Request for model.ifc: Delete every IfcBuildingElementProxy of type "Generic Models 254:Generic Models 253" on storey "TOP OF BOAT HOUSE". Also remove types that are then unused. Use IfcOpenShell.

First a look at what the model holds.

```python
import ifcopenshell
import ifcopenshell.util.element

model = ifcopenshell.open("model.ifc")
print(model.schema)
storey = next(s for s in model.by_type("IfcBuildingStorey") if s.Name == "TOP OF BOAT HOUSE")
proxies = [e for e in ifcopenshell.util.element.get_decomposition(storey) if e.is_a("IfcBuildingElementProxy")]
seen = {}
for e in proxies:
    element_type = ifcopenshell.util.element.get_type(e)
    name = element_type.Name if element_type not in (None, e) else None
    seen[name] = seen.get(name, 0) + 1
for name, count in sorted(seen.items(), key=str):
    print(count, "x", name)
```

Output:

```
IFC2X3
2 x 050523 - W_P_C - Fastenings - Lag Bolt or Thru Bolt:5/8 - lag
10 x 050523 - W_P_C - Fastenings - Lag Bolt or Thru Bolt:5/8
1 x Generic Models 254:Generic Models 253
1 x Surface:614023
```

```python
import ifcopenshell
import ifcopenshell.api.root
import ifcopenshell.util.element

model = ifcopenshell.open("model.ifc")

storey = next(s for s in model.by_type("IfcBuildingStorey") if s.Name == "TOP OF BOAT HOUSE")
proxies = [e for e in ifcopenshell.util.element.get_decomposition(storey) if e.is_a("IfcBuildingElementProxy")]
targets = [e for e in proxies if (t := ifcopenshell.util.element.get_type(e)) not in (None, e) and t.Name == "Generic Models 254:Generic Models 253"]
types = {ifcopenshell.util.element.get_type(e) for e in targets} - {None, *targets}

for e in targets:
    ifcopenshell.api.root.remove_product(model, product=e)
print(len(targets), "removed")

unused = [t for t in types if not ifcopenshell.util.element.get_types(t)]
for t in unused:
    ifcopenshell.api.root.remove_product(model, product=t)
print(len(unused), "unused types removed")

model.write("model-out.ifc")
```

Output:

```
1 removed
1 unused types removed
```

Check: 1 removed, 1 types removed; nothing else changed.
